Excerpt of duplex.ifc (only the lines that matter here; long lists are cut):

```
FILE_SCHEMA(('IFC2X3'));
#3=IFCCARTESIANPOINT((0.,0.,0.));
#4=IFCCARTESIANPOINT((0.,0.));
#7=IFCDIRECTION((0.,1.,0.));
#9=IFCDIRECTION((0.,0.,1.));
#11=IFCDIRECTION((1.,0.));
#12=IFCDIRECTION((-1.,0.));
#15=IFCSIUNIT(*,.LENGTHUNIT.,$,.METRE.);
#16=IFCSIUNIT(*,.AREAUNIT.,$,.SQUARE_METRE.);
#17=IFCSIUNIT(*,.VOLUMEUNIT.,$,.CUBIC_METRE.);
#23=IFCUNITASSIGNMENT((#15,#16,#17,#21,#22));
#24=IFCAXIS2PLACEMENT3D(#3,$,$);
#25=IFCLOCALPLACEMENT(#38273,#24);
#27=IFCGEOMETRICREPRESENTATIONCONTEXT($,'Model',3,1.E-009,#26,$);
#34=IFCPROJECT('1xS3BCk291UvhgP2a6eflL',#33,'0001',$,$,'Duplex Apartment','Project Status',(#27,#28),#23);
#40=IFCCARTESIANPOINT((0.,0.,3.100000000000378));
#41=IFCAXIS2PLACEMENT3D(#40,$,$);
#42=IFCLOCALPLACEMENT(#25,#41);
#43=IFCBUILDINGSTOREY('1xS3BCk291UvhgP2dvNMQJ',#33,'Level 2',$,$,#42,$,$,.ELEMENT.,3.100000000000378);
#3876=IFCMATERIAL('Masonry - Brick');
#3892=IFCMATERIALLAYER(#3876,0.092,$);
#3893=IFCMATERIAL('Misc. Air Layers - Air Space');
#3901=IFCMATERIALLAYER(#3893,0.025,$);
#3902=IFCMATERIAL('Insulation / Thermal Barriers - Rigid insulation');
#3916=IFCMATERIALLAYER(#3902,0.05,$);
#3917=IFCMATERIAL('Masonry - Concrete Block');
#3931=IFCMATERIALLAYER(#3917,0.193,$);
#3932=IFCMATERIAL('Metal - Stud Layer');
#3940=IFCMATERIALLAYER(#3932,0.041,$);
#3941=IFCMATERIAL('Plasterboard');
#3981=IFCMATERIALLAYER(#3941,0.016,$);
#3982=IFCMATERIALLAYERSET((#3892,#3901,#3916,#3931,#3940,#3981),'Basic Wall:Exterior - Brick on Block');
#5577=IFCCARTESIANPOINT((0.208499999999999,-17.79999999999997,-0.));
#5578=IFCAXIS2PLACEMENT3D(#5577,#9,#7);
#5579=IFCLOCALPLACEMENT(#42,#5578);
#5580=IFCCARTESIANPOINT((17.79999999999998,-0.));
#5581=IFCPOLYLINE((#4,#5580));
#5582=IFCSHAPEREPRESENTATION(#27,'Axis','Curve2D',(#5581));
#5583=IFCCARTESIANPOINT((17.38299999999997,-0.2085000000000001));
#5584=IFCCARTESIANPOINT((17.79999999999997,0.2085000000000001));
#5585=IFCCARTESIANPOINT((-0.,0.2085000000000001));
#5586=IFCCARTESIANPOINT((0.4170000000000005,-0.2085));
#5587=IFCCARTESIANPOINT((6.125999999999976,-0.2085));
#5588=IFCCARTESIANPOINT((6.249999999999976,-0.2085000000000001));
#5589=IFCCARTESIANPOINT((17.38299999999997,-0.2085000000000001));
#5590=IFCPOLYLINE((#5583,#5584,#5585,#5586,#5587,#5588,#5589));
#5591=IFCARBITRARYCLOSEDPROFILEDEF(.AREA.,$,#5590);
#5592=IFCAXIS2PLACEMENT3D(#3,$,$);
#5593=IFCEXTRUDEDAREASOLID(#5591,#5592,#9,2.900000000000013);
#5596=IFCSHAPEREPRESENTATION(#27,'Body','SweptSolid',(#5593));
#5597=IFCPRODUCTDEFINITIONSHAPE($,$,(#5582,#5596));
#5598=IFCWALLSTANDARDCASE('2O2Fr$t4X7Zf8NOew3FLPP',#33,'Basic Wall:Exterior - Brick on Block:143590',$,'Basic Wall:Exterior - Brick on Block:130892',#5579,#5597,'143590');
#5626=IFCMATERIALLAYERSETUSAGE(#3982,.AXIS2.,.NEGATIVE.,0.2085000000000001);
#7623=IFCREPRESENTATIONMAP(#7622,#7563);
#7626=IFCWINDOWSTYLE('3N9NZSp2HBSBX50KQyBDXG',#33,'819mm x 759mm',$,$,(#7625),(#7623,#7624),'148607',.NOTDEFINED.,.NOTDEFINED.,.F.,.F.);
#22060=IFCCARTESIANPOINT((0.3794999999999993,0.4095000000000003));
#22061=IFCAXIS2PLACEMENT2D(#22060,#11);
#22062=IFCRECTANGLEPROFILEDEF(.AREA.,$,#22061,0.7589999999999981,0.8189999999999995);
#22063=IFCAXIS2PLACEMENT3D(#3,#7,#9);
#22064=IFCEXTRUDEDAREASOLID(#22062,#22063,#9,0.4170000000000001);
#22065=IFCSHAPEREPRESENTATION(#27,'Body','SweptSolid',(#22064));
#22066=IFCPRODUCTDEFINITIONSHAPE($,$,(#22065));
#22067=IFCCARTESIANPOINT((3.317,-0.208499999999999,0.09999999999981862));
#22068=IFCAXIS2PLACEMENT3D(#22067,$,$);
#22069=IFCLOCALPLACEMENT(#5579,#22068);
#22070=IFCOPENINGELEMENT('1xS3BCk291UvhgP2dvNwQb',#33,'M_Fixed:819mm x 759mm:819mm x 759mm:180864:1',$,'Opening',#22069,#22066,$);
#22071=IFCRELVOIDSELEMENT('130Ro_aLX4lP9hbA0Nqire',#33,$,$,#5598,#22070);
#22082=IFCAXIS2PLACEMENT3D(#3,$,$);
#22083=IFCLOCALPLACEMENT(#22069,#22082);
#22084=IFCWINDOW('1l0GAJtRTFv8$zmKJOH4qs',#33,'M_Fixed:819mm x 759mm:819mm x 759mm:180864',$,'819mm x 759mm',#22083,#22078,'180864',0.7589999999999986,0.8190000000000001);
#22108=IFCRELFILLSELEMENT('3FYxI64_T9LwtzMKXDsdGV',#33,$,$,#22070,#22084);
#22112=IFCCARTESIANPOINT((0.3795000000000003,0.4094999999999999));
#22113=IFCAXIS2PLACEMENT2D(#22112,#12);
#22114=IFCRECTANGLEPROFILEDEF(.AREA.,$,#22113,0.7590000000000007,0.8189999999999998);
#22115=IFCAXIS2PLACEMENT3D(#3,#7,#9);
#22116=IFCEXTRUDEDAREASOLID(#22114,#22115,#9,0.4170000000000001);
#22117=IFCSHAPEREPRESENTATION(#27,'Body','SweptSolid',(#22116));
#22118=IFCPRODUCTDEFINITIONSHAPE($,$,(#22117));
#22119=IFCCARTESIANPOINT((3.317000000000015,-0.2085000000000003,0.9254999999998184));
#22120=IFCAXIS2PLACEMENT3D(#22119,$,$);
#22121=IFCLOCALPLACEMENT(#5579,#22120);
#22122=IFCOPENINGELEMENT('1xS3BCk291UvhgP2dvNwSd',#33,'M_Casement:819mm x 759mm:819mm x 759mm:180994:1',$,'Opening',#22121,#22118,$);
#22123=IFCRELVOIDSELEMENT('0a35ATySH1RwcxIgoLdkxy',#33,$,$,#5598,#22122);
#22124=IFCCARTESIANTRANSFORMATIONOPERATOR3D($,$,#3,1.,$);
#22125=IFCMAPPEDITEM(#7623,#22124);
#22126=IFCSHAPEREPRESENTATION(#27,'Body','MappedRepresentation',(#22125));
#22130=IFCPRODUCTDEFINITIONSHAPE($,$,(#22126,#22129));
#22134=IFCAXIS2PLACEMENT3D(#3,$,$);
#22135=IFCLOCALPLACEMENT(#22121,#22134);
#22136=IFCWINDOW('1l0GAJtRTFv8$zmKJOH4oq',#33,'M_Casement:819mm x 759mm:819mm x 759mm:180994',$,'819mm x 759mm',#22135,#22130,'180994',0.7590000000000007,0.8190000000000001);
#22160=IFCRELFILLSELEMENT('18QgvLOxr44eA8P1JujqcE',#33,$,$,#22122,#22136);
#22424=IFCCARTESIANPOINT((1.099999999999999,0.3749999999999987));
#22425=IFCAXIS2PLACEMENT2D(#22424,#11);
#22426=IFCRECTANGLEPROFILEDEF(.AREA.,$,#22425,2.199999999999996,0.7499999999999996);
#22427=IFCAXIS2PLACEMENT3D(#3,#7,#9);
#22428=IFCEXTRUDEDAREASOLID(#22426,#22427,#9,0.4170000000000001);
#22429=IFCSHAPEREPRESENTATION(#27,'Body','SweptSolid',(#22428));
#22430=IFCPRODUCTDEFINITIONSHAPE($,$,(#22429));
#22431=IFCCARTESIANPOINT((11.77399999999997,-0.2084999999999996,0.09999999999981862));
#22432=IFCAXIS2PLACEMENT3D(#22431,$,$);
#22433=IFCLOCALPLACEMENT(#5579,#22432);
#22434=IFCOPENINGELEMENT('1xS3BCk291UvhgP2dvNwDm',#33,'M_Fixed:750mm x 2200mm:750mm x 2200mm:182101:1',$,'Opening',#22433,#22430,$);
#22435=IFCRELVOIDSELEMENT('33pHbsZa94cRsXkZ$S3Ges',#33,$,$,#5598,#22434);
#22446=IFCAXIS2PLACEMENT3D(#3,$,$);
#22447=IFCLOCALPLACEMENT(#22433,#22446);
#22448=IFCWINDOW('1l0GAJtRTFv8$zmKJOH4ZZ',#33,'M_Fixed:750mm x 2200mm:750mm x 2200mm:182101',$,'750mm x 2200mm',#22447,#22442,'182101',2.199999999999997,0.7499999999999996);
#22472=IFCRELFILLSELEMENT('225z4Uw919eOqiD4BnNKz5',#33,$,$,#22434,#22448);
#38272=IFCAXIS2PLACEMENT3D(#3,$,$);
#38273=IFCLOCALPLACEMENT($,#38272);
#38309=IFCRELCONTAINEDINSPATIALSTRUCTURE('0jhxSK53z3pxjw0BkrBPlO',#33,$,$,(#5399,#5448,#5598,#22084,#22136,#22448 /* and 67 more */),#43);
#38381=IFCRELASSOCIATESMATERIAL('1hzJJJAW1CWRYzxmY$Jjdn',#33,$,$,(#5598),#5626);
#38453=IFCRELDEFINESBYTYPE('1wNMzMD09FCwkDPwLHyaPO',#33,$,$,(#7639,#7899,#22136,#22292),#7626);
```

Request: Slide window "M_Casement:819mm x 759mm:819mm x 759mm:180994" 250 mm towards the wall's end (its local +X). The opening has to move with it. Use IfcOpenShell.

```python
import ifcopenshell
import ifcopenshell.api.geometry
import ifcopenshell.util.placement

model = ifcopenshell.open("duplex.ifc")

window = model.by_guid("1l0GAJtRTFv8$zmKJOH4oq")
opening = window.FillsVoids[0].RelatingOpeningElement
wall = opening.VoidsElements[0].RelatingBuildingElement

wall_matrix = ifcopenshell.util.placement.get_local_placement(wall.ObjectPlacement)
shift = wall_matrix[:3, 0] * 0.25
before = ifcopenshell.util.placement.get_local_placement(window.ObjectPlacement)[:3, 3].copy()

# The window is placed relative to its opening, so it follows when the opening moves.
matrix = ifcopenshell.util.placement.get_local_placement(opening.ObjectPlacement)
matrix[:3, 3] += shift
ifcopenshell.api.geometry.edit_object_placement(
    model, product=opening, matrix=matrix, is_si=False, should_transform_children=True
)

after = ifcopenshell.util.placement.get_local_placement(window.ObjectPlacement)[:3, 3]
print("window moved by", (after - before).round(3) + 0.0)

model.write("duplex_updated.ifc")
```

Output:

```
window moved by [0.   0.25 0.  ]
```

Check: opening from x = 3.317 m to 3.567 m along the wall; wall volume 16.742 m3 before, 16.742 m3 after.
